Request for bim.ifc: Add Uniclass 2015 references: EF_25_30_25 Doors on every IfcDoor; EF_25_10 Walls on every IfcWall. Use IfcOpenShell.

First a look at what the model holds.

```python
import ifcopenshell

model = ifcopenshell.open("bim.ifc")
print(model.schema)
print("classifications:", [c.Name for c in model.by_type("IfcClassification")])
for ifc_class in ("IfcDoor", "IfcRoof", "IfcStair", "IfcWall", "IfcWindow"):
    print(ifc_class, len(model.by_type(ifc_class)))
```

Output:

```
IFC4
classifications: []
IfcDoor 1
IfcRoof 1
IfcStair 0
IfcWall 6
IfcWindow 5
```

```python
import ifcopenshell
import ifcopenshell.api.classification

model = ifcopenshell.open("bim.ifc")

system = ifcopenshell.api.classification.add_classification(model, classification="Uniclass 2015")

codes = {
    "IfcDoor": ("EF_25_30_25", "Doors"),
    "IfcWall": ("EF_25_10", "Walls"),
}
for ifc_class, (code, name) in codes.items():
    products = model.by_type(ifc_class)
    ifcopenshell.api.classification.add_reference(
        model, products=products, classification=system, identification=code, name=name
    )
    print(code, len(products))

model.write("bim_rev.ifc")
```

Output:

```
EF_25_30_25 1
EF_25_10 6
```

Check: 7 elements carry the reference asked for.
